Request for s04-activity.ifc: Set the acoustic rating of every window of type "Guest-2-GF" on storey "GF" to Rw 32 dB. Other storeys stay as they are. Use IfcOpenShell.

First a look at what the model holds.

```python
import ifcopenshell
import ifcopenshell.util.element

model = ifcopenshell.open("s04-activity.ifc")
print(model.schema)
storey = next(s for s in model.by_type("IfcBuildingStorey") if s.Name == "GF")
windows = [e for e in ifcopenshell.util.element.get_decomposition(storey) if e.is_a("IfcWindow")]
seen = {}
for e in windows:
    element_type = ifcopenshell.util.element.get_type(e)
    key = (element_type.Name if element_type != e and element_type else None, ifcopenshell.util.element.get_pset(e, "Pset_WindowCommon", "AcousticRating"))
    seen[key] = seen.get(key, 0) + 1
for (name, value), count in sorted(seen.items(), key=str):
    print(count, "x", name, "|", value)
```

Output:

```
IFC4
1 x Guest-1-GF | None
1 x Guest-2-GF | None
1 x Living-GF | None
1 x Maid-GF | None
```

```python
import ifcopenshell
import ifcopenshell.api.pset
import ifcopenshell.util.element

model = ifcopenshell.open("s04-activity.ifc")

storey = next(s for s in model.by_type("IfcBuildingStorey") if s.Name == "GF")
windows = [e for e in ifcopenshell.util.element.get_decomposition(storey) if e.is_a("IfcWindow")]

count = 0
for e in windows:
    element_type = ifcopenshell.util.element.get_type(e)
    if element_type in (None, e) or element_type.Name != "Guest-2-GF":
        continue
    # add_pset returns the element's existing set when there is one.
    pset = ifcopenshell.api.pset.add_pset(model, product=e, name="Pset_WindowCommon")
    ifcopenshell.api.pset.edit_pset(model, pset=pset, properties={"AcousticRating": "Rw 32 dB"})
    count += 1

print(count, "windows updated")

model.write("s04-activity-out.ifc")
```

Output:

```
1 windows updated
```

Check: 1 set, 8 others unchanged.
